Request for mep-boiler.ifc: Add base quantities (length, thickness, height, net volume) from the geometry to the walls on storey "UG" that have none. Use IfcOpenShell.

First a look at what the model holds.

```python
import ifcopenshell
import ifcopenshell.util.element
import ifcopenshell.util.unit

model = ifcopenshell.open("mep-boiler.ifc")
print(model.schema)
for unit_type in ("LENGTHUNIT", "AREAUNIT", "VOLUMEUNIT"):
    print(unit_type, ifcopenshell.util.unit.calculate_unit_scale(model, unit_type))
storey = next(s for s in model.by_type("IfcBuildingStorey") if s.Name == "UG")
walls = [e for e in ifcopenshell.util.element.get_decomposition(storey) if e.is_a("IfcWall")]
for e in sorted(walls, key=lambda e: e.id()):
    print(e.id(), e.is_a(), e.Name, list(ifcopenshell.util.element.get_psets(e, qtos_only=True)), sep=" | ")
```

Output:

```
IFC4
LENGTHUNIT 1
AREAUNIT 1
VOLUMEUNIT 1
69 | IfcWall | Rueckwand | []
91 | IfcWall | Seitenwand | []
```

```python
import ifcopenshell
import ifcopenshell.api.pset
import ifcopenshell.geom
import ifcopenshell.util.element
import ifcopenshell.util.shape
import ifcopenshell.util.unit

model = ifcopenshell.open("mep-boiler.ifc")
unit_scale = ifcopenshell.util.unit.calculate_unit_scale(model)
volume_scale = ifcopenshell.util.unit.calculate_unit_scale(model, "VOLUMEUNIT")
settings = ifcopenshell.geom.settings()

storey = next(s for s in model.by_type("IfcBuildingStorey") if s.Name == "UG")
walls = [e for e in ifcopenshell.util.element.get_decomposition(storey) if e.is_a("IfcWall")]

for e in sorted(walls, key=lambda e: e.id()):
    if ifcopenshell.util.element.get_psets(e, qtos_only=True, should_inherit=False):
        continue
    # Geometry comes back in metres, in the element's own axes.
    shape = ifcopenshell.geom.create_shape(settings, e)
    values = {
        "Length": ifcopenshell.util.shape.get_x(shape.geometry) / unit_scale,
        "Width": ifcopenshell.util.shape.get_y(shape.geometry) / unit_scale,
        "Height": ifcopenshell.util.shape.get_z(shape.geometry) / unit_scale,
        "NetVolume": ifcopenshell.util.shape.get_volume(shape.geometry) / volume_scale,
    }
    qto = ifcopenshell.api.pset.add_qto(model, product=e, name="Qto_WallBaseQuantities")
    ifcopenshell.api.pset.edit_qto(model, qto=qto, properties=values)
    print(e.id(), {k: round(v, 3) for k, v in values.items()})

model.write("mep-boiler_updated.ifc")
```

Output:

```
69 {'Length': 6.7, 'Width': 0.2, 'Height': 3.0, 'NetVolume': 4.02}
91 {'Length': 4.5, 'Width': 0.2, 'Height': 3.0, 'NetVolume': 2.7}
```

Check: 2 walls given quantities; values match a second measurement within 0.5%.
